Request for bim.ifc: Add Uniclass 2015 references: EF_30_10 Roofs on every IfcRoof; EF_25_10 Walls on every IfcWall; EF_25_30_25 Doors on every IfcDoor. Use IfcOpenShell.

First a look at what the model holds.

```python
import ifcopenshell

model = ifcopenshell.open("bim.ifc")
print(model.schema)
print("classifications:", [c.Name for c in model.by_type("IfcClassification")])
for ifc_class in ("IfcDoor", "IfcRoof", "IfcStair", "IfcWall", "IfcWindow"):
    print(ifc_class, len(model.by_type(ifc_class)))
```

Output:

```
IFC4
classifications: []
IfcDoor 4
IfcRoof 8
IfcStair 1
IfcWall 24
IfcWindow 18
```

```python
import ifcopenshell
import ifcopenshell.api.classification

model = ifcopenshell.open("bim.ifc")

system = ifcopenshell.api.classification.add_classification(model, classification="Uniclass 2015")

codes = {
    "IfcRoof": ("EF_30_10", "Roofs"),
    "IfcWall": ("EF_25_10", "Walls"),
    "IfcDoor": ("EF_25_30_25", "Doors"),
}
for ifc_class, (code, name) in codes.items():
    products = model.by_type(ifc_class)
    ifcopenshell.api.classification.add_reference(
        model, products=products, classification=system, identification=code, name=name
    )
    print(code, len(products))

model.write("bim_updated.ifc")
```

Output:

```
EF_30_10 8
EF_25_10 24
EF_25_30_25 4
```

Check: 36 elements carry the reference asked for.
